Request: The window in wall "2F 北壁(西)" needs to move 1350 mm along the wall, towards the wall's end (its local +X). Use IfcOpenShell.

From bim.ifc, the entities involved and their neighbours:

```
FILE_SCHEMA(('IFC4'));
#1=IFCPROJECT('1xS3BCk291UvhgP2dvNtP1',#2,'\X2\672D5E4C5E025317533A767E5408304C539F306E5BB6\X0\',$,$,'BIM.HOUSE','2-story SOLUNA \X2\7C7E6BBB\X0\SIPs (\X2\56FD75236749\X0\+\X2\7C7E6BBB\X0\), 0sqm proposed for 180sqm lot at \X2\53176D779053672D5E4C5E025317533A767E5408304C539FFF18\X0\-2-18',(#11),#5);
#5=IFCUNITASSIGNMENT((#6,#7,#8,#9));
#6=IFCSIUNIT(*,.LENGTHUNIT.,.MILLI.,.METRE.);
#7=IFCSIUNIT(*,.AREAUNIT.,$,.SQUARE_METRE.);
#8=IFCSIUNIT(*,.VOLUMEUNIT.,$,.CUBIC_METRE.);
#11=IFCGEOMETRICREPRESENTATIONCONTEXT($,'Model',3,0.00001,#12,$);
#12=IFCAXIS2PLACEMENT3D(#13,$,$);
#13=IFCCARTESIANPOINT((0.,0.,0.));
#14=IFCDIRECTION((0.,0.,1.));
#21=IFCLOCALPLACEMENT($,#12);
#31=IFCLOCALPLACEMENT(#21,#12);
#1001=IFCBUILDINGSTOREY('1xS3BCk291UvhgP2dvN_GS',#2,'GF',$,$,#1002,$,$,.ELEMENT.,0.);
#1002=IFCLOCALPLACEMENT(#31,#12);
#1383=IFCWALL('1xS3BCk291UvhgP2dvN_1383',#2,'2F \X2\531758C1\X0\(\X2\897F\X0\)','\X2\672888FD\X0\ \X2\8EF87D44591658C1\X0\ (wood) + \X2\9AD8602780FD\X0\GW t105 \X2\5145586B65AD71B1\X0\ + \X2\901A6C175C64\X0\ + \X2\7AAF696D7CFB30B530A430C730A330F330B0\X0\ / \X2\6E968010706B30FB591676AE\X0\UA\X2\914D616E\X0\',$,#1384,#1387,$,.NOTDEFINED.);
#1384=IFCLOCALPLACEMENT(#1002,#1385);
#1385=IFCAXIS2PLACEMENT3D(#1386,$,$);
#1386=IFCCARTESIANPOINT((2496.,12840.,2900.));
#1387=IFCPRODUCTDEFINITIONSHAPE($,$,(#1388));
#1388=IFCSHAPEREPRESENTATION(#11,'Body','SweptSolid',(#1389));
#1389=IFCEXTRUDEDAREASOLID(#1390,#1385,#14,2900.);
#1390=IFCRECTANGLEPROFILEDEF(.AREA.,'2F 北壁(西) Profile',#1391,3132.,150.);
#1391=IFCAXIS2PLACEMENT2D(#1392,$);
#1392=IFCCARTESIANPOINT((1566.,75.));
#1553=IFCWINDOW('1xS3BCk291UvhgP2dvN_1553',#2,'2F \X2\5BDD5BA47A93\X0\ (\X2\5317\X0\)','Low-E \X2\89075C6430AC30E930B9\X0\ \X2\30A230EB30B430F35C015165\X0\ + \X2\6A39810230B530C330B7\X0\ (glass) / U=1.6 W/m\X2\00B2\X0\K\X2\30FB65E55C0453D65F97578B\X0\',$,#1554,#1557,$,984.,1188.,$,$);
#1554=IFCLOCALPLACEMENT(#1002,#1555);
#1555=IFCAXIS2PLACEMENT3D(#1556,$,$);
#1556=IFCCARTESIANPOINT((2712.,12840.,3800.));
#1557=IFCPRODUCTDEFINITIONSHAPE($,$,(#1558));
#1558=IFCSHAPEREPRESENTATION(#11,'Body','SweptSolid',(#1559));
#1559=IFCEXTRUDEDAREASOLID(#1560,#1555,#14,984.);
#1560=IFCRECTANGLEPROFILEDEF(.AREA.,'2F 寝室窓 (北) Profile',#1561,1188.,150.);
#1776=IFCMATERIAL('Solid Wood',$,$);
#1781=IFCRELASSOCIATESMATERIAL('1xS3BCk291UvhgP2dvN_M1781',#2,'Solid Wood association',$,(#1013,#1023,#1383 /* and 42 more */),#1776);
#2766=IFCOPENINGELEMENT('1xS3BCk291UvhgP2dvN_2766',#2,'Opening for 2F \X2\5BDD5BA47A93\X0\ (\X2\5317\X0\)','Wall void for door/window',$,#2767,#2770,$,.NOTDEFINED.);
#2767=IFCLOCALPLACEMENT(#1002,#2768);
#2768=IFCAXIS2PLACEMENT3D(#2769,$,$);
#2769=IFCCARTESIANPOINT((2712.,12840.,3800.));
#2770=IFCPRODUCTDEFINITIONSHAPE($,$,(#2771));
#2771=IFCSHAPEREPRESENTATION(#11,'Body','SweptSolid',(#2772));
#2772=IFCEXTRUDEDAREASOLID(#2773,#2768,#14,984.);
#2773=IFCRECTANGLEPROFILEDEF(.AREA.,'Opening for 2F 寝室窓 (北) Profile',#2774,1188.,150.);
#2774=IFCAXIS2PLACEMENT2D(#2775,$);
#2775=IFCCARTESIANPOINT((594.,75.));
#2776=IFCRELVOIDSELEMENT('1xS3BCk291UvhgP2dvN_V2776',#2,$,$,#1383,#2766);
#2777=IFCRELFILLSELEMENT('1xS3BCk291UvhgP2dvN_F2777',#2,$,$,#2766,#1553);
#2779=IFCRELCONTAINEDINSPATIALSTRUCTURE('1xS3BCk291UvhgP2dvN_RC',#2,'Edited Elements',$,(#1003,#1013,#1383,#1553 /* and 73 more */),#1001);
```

```python
import ifcopenshell
import ifcopenshell.api.geometry
import ifcopenshell.util.placement
import ifcopenshell.util.unit

model = ifcopenshell.open("bim.ifc")
unit_scale = ifcopenshell.util.unit.calculate_unit_scale(model)

window = model.by_id(1553)
opening = window.FillsVoids[0].RelatingOpeningElement
wall = opening.VoidsElements[0].RelatingBuildingElement

wall_matrix = ifcopenshell.util.placement.get_local_placement(wall.ObjectPlacement)
shift = wall_matrix[:3, 0] * 1.35 / unit_scale
before = ifcopenshell.util.placement.get_local_placement(window.ObjectPlacement)[:3, 3].copy()

# The window is not placed relative to its opening, so move both.
for product in (opening, window):
    matrix = ifcopenshell.util.placement.get_local_placement(product.ObjectPlacement)
    matrix[:3, 3] += shift
    ifcopenshell.api.geometry.edit_object_placement(model, product=product, matrix=matrix, is_si=False)

after = ifcopenshell.util.placement.get_local_placement(window.ObjectPlacement)[:3, 3]
print("window moved by", (after - before).round(3) + 0.0)

model.write("bim_updated.ifc")
```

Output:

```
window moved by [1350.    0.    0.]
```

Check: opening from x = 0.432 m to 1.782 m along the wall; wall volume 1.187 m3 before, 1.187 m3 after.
